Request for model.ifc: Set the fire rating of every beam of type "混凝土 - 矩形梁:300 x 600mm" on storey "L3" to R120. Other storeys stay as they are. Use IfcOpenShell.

First a look at what the model holds.

```python
import ifcopenshell
import ifcopenshell.util.element

model = ifcopenshell.open("model.ifc")
print(model.schema)
storey = next(s for s in model.by_type("IfcBuildingStorey") if s.Name == "L3")
beams = [e for e in ifcopenshell.util.element.get_decomposition(storey) if e.is_a("IfcBeam")]
seen = {}
for e in beams:
    element_type = ifcopenshell.util.element.get_type(e)
    key = (element_type.Name if element_type != e and element_type else None, ifcopenshell.util.element.get_pset(e, "Pset_BeamCommon", "FireRating"))
    seen[key] = seen.get(key, 0) + 1
for (name, value), count in sorted(seen.items(), key=str):
    print(count, "x", name, "|", value)
```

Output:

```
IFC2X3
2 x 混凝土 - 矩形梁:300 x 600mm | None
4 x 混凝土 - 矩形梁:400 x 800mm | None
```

```python
import ifcopenshell
import ifcopenshell.api.pset
import ifcopenshell.util.element

model = ifcopenshell.open("model.ifc")

storey = next(s for s in model.by_type("IfcBuildingStorey") if s.Name == "L3")
beams = [e for e in ifcopenshell.util.element.get_decomposition(storey) if e.is_a("IfcBeam")]

count = 0
for e in beams:
    element_type = ifcopenshell.util.element.get_type(e)
    if element_type in (None, e) or element_type.Name != "混凝土 - 矩形梁:300 x 600mm":
        continue
    # add_pset returns the element's existing set when there is one.
    pset = ifcopenshell.api.pset.add_pset(model, product=e, name="Pset_BeamCommon")
    ifcopenshell.api.pset.edit_pset(model, pset=pset, properties={"FireRating": "R120"})
    count += 1

print(count, "beams updated")

model.write("model_updated.ifc")
```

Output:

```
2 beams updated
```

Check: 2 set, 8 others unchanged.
